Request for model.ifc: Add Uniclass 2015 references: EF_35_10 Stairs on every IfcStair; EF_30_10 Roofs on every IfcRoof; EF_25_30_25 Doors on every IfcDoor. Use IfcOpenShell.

First a look at what the model holds.

```python
import ifcopenshell

model = ifcopenshell.open("model.ifc")
print(model.schema)
print("classifications:", [c.Name for c in model.by_type("IfcClassification")])
for ifc_class in ("IfcDoor", "IfcRoof", "IfcStair", "IfcWall", "IfcWindow"):
    print(ifc_class, len(model.by_type(ifc_class)))
```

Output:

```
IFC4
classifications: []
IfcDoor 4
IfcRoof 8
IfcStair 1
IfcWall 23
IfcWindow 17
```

```python
import ifcopenshell
import ifcopenshell.api.classification

model = ifcopenshell.open("model.ifc")

system = ifcopenshell.api.classification.add_classification(model, classification="Uniclass 2015")

codes = {
    "IfcStair": ("EF_35_10", "Stairs"),
    "IfcRoof": ("EF_30_10", "Roofs"),
    "IfcDoor": ("EF_25_30_25", "Doors"),
}
for ifc_class, (code, name) in codes.items():
    products = model.by_type(ifc_class)
    ifcopenshell.api.classification.add_reference(
        model, products=products, classification=system, identification=code, name=name
    )
    print(code, len(products))

model.write("model-out.ifc")
```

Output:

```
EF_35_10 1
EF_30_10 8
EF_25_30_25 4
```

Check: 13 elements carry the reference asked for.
